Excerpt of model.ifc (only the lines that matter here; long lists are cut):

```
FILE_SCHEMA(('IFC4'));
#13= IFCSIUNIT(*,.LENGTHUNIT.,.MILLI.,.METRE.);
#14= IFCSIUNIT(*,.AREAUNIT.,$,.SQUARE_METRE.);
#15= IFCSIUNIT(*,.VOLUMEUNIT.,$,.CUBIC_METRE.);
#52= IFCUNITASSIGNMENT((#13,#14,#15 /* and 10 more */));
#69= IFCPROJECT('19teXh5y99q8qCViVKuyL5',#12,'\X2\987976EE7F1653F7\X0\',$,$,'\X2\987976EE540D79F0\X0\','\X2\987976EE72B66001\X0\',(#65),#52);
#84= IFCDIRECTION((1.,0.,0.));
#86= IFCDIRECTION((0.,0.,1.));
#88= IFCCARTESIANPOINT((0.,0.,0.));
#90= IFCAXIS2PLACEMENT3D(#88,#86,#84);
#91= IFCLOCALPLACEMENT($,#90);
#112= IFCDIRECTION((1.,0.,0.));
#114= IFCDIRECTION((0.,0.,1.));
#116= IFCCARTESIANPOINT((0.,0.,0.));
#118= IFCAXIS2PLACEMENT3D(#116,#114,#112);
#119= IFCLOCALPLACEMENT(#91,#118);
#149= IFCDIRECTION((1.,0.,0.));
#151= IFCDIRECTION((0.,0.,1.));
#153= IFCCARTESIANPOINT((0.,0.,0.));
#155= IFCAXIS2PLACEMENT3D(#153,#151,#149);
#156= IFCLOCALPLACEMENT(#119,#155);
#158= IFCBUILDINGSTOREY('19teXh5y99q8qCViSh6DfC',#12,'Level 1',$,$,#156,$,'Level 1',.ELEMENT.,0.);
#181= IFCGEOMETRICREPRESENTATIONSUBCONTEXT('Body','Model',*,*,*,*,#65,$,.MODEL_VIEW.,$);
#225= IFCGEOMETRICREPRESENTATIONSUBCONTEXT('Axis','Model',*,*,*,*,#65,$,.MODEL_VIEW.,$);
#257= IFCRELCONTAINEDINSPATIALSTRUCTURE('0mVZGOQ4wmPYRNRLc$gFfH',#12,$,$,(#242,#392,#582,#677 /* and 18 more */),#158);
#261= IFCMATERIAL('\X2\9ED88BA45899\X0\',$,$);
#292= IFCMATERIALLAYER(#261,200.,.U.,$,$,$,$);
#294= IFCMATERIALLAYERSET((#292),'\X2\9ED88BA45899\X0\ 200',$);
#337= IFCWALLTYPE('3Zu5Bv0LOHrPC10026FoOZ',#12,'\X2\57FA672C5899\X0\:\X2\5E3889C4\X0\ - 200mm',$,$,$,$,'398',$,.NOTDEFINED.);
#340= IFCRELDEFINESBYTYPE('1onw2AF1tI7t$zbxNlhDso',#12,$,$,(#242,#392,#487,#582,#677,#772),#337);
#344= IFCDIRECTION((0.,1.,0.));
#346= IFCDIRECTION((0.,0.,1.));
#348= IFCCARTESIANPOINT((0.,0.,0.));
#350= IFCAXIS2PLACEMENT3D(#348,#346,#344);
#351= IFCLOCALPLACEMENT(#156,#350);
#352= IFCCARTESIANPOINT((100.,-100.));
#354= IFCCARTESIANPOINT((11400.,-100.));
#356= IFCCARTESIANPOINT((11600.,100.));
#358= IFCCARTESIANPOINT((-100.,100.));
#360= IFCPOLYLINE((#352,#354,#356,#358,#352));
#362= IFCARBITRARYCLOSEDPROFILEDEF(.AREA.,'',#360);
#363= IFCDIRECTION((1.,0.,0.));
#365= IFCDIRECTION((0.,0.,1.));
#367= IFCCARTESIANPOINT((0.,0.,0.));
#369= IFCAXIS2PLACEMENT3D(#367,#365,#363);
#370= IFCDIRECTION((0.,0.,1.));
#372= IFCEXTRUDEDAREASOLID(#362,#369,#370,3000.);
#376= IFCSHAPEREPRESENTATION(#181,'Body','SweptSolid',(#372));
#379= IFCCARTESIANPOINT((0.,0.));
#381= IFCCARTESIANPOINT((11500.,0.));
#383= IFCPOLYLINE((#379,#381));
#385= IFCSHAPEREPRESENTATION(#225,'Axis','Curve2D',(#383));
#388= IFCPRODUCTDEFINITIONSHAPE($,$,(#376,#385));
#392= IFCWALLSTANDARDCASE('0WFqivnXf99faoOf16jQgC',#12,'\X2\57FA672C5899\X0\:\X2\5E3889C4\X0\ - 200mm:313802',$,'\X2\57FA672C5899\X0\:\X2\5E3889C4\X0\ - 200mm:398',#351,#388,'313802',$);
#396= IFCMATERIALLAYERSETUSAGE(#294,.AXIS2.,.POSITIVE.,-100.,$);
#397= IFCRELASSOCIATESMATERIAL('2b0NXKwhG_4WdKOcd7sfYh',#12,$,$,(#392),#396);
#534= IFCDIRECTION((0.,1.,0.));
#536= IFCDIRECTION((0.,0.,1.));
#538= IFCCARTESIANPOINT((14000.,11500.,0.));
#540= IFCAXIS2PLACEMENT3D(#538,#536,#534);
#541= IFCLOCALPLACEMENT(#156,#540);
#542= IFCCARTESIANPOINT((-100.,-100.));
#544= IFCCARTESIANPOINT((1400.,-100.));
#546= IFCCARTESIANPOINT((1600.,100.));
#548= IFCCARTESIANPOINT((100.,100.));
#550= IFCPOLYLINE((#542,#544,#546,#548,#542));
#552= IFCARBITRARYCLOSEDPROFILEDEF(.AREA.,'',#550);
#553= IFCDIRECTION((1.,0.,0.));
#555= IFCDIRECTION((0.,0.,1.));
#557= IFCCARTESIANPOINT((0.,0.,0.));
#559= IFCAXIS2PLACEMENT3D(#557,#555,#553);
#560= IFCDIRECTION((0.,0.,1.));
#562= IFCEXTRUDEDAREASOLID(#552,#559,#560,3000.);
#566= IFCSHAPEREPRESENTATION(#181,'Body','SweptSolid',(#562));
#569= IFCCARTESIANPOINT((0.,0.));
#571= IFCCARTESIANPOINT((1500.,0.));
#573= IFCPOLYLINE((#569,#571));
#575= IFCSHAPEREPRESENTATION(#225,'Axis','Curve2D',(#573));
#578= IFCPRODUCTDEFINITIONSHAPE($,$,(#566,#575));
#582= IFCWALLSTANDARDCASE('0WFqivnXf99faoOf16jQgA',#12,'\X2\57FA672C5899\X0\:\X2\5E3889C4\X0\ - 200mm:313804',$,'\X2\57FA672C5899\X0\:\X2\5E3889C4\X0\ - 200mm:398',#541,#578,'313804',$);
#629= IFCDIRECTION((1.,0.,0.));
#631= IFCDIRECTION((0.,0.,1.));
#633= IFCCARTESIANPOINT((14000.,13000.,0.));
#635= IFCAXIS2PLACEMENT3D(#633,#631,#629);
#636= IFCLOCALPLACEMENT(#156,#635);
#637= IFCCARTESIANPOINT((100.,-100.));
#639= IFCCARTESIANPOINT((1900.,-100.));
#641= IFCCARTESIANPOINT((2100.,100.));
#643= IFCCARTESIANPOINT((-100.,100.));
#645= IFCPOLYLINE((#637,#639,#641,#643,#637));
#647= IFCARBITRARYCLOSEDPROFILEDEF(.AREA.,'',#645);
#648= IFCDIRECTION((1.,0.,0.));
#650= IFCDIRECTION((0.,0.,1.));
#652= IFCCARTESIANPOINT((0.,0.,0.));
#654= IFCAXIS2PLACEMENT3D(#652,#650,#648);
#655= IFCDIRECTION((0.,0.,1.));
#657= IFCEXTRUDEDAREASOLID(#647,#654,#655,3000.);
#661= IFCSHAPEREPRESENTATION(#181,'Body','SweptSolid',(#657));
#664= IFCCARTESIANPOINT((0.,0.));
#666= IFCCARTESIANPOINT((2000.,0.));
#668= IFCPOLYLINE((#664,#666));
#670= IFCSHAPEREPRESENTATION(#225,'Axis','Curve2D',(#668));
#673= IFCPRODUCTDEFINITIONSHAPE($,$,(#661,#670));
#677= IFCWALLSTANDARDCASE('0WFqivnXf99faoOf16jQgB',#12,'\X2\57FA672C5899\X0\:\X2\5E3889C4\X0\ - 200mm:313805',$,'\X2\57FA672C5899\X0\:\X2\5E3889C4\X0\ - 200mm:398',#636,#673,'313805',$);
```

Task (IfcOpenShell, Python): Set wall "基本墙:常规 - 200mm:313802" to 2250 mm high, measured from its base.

```python
import ifcopenshell
import ifcopenshell.geom
import ifcopenshell.util.representation
import ifcopenshell.util.shape

model = ifcopenshell.open("model.ifc")
settings = ifcopenshell.geom.settings()


def volume(element):
    """Net volume in cubic metres, openings subtracted."""
    shape = ifcopenshell.geom.create_shape(settings, element)
    return ifcopenshell.util.shape.get_volume(shape.geometry)


wall = model.by_id(392)
before = volume(wall)

body = ifcopenshell.util.representation.get_representation(wall, "Model", "Body")
solid = body.Items[0]
old_height = solid.Depth
solid.Depth = 2250.0
after = volume(wall)

print(f"height {old_height:g} -> {solid.Depth:g}, volume {before:.3f} -> {after:.3f} m3")

model.write("model-out.ifc")
```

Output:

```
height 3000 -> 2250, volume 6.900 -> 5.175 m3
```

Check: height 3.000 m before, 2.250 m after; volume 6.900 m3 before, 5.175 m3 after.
